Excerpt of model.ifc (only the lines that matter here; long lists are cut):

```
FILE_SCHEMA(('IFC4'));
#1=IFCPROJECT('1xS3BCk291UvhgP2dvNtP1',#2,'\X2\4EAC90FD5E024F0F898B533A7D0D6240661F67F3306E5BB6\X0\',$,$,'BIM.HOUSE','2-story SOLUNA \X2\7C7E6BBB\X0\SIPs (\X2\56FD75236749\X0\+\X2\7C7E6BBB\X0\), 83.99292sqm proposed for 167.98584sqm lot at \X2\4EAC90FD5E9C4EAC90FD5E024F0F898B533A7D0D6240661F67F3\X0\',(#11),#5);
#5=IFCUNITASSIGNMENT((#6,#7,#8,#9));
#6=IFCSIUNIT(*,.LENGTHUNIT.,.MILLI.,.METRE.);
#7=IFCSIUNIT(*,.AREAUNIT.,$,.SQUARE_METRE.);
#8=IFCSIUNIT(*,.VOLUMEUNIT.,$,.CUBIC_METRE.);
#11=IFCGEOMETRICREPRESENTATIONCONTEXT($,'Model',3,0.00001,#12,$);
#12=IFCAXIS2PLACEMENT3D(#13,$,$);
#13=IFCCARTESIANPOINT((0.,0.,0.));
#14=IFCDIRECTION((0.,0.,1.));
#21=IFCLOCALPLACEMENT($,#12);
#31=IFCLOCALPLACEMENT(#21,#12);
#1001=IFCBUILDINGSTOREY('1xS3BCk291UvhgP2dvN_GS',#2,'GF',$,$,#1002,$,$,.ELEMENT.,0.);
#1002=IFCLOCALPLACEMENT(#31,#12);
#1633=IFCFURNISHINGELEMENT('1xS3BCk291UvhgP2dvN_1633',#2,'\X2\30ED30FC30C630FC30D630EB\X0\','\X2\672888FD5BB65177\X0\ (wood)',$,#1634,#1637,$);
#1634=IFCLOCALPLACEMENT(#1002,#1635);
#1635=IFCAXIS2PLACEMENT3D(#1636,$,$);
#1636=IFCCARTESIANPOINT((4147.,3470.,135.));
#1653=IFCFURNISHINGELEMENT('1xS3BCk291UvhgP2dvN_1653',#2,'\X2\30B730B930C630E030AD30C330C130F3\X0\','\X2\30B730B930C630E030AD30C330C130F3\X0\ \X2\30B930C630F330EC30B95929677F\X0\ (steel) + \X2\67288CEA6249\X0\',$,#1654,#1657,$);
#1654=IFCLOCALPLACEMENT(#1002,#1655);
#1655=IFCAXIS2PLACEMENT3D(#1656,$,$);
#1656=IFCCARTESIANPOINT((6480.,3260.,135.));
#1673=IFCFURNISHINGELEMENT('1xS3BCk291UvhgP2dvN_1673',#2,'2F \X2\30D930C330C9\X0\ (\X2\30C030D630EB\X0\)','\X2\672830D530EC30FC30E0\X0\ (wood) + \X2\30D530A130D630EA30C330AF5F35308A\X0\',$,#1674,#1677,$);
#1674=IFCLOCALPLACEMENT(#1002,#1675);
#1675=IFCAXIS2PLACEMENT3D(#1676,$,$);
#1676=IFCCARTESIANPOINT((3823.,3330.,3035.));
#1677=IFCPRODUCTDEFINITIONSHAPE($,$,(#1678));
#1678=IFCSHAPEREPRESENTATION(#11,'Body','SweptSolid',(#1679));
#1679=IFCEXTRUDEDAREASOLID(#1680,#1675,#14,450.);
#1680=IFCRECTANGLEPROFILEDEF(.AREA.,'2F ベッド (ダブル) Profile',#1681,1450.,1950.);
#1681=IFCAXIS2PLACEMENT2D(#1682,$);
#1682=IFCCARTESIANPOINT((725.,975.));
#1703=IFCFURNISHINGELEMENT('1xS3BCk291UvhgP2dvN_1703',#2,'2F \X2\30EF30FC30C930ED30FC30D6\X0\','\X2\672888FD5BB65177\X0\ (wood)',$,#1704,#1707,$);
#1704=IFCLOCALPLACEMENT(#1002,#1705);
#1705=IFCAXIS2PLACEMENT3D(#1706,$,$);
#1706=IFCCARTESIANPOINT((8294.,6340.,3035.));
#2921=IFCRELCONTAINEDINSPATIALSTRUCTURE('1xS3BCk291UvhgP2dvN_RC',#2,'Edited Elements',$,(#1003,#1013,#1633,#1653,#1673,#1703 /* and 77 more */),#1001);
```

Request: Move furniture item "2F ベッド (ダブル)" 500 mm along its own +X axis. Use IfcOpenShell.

```python
import ifcopenshell
import ifcopenshell.api.geometry
import ifcopenshell.util.placement
import ifcopenshell.util.unit

model = ifcopenshell.open("model.ifc")
unit_scale = ifcopenshell.util.unit.calculate_unit_scale(model)

item = model.by_guid("1xS3BCk291UvhgP2dvN_1673")
matrix = ifcopenshell.util.placement.get_local_placement(item.ObjectPlacement)
matrix[:3, 3] += matrix[:3, 0] * 0.5 / unit_scale
ifcopenshell.api.geometry.edit_object_placement(model, product=item, matrix=matrix, is_si=False)

print(ifcopenshell.util.placement.get_local_placement(item.ObjectPlacement).round(3) + 0.0)

model.write("model_rev.ifc")
```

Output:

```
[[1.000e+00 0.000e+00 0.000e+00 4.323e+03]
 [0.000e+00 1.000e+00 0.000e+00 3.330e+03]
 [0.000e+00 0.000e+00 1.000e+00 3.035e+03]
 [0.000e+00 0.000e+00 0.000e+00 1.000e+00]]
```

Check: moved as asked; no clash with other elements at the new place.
